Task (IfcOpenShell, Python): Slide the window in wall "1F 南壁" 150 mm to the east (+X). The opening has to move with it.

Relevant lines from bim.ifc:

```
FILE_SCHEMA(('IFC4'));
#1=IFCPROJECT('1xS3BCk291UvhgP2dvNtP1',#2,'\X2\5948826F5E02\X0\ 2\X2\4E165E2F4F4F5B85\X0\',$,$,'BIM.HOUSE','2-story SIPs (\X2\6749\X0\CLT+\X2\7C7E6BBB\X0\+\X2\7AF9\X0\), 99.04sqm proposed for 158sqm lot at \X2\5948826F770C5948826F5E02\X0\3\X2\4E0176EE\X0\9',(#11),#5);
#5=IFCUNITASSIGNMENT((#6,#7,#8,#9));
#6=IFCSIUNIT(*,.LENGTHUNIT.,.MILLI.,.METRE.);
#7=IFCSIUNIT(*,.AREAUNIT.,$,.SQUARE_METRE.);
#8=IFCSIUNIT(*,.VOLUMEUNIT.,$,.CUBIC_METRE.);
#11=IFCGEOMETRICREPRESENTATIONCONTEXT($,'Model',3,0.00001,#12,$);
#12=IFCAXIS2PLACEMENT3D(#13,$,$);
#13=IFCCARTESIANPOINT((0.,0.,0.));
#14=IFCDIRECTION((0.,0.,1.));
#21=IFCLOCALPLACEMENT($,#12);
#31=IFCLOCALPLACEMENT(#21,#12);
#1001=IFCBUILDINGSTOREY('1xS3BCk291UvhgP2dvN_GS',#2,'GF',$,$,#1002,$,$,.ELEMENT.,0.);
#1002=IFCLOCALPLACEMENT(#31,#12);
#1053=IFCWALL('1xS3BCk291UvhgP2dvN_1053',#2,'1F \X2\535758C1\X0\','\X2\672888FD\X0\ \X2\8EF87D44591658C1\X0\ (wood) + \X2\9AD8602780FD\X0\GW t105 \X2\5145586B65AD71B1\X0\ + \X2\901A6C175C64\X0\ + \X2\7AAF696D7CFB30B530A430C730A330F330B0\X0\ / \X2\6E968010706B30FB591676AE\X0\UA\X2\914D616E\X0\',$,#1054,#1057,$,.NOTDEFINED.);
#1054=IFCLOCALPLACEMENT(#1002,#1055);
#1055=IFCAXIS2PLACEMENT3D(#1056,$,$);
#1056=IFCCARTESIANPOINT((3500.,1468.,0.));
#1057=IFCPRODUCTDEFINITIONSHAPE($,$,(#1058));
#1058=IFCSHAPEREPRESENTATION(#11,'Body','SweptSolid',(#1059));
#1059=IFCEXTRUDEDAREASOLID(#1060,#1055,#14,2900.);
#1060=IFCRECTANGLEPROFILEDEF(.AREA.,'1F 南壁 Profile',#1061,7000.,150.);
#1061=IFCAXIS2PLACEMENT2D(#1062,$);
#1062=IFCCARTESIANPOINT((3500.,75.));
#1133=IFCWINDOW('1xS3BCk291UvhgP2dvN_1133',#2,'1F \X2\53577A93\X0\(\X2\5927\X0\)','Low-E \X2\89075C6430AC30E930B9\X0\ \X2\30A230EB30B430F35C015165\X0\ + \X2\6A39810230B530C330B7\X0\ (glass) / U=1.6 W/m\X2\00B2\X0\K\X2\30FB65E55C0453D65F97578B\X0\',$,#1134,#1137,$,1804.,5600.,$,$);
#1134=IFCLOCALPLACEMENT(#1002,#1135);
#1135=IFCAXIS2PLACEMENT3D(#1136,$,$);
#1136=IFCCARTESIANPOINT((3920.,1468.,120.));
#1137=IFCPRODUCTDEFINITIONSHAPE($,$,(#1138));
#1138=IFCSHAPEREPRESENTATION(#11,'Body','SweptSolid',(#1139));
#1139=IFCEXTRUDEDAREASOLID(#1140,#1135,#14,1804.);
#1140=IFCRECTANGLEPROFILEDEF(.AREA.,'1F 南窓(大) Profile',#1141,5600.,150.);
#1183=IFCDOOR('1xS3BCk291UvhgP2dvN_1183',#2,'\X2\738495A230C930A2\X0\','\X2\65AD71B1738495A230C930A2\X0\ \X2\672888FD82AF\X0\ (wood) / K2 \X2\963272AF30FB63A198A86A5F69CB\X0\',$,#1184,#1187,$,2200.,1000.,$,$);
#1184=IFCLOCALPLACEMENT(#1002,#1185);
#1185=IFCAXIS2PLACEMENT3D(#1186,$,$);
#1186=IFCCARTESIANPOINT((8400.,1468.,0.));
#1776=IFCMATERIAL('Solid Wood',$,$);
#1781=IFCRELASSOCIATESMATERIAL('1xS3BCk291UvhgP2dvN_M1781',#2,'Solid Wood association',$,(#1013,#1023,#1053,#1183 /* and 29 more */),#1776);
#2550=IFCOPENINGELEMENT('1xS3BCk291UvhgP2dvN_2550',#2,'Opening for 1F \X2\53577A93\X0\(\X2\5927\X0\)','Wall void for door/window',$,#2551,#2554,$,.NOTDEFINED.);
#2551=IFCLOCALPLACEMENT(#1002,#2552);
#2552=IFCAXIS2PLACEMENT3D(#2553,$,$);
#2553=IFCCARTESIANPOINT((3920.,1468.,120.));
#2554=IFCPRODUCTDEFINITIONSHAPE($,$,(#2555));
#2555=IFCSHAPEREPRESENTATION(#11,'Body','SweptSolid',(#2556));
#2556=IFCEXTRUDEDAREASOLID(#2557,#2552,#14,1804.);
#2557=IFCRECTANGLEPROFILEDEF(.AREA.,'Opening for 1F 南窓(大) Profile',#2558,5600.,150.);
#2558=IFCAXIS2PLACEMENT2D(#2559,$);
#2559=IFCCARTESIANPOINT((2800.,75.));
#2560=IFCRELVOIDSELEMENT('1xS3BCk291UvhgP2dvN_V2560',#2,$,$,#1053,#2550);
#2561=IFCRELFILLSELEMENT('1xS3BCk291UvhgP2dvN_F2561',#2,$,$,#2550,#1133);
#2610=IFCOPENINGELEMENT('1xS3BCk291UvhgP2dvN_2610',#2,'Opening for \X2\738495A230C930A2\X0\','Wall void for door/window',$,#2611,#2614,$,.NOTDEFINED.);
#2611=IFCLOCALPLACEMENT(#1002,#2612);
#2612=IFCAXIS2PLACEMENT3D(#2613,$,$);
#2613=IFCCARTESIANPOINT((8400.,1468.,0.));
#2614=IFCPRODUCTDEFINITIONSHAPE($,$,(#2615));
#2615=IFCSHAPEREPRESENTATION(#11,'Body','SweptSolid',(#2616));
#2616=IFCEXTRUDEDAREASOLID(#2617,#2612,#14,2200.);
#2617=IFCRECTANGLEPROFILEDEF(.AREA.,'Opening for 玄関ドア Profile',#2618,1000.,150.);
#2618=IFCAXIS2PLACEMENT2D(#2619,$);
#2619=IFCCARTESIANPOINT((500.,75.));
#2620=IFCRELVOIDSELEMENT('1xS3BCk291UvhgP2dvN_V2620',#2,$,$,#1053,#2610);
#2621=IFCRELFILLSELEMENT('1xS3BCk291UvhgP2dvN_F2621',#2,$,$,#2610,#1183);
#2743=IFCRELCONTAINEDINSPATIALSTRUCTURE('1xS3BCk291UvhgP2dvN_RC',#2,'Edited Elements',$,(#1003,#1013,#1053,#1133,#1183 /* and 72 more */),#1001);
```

```python
import ifcopenshell
import ifcopenshell.api.geometry
import ifcopenshell.util.placement

model = ifcopenshell.open("bim.ifc")

window = model.by_id(1133)
opening = window.FillsVoids[0].RelatingOpeningElement
wall = opening.VoidsElements[0].RelatingBuildingElement

wall_matrix = ifcopenshell.util.placement.get_local_placement(wall.ObjectPlacement)
shift = wall_matrix[:3, 0] * 150.0
before = ifcopenshell.util.placement.get_local_placement(window.ObjectPlacement)[:3, 3].copy()

# The window is not placed relative to its opening, so move both.
for product in (opening, window):
    matrix = ifcopenshell.util.placement.get_local_placement(product.ObjectPlacement)
    matrix[:3, 3] += shift
    ifcopenshell.api.geometry.edit_object_placement(model, product=product, matrix=matrix, is_si=False)

after = ifcopenshell.util.placement.get_local_placement(window.ObjectPlacement)[:3, 3]
print("window moved by", (after - before).round(3) + 0.0)

model.write("bim_updated.ifc")
```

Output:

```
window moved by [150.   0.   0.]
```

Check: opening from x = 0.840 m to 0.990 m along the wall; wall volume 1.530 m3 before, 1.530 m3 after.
